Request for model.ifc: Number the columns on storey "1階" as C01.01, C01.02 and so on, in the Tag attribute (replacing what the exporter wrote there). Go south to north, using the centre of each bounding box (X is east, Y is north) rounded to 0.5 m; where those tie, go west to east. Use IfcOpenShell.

First a look at what the model holds.

```python
import ifcopenshell
import ifcopenshell.util.element
import ifcopenshell.util.placement

model = ifcopenshell.open("model.ifc")
print(model.schema)
storey = next(s for s in model.by_type("IfcBuildingStorey") if s.Name == "1階")
columns = [e for e in ifcopenshell.util.element.get_decomposition(storey) if e.is_a("IfcColumn")]
for e in sorted(columns, key=lambda e: e.id()):
    origin = ifcopenshell.util.placement.get_local_placement(e.ObjectPlacement)[:3, 3]
    print(e.id(), e.Tag, e.Name, origin.round(2) + 0.0, sep=" | ")
```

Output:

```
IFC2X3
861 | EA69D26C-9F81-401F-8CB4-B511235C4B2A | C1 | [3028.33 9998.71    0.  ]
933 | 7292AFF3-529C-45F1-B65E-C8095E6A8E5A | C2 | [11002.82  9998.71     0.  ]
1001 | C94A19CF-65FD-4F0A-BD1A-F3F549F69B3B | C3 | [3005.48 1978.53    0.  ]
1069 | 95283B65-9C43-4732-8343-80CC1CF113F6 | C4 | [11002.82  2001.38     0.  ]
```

```python
import ifcopenshell
import ifcopenshell.geom
import ifcopenshell.util.element
import ifcopenshell.util.shape

model = ifcopenshell.open("model.ifc")
settings = ifcopenshell.geom.settings()
settings.set("use-world-coords", True)


def centre(element):
    shape = ifcopenshell.geom.create_shape(settings, element)
    return ifcopenshell.util.shape.get_bbox_centroid(shape.geometry)


storey = next(s for s in model.by_type("IfcBuildingStorey") if s.Name == "1階")
columns = [e for e in ifcopenshell.util.element.get_decomposition(storey) if e.is_a("IfcColumn")]

# Insertion points can sit at a corner or the storey origin, so sort by the geometry (in metres).
centres = {e: centre(e) for e in columns}
columns.sort(key=lambda e: (round(centres[e][1] / 0.5), centres[e][0]))

for i, e in enumerate(columns, start=1):
    number = f"C01.{i:02d}"
    e.Tag = number
    print(e.id(), number)

model.write("model_updated.ifc")
```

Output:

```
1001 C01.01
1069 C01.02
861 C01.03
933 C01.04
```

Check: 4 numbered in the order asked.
